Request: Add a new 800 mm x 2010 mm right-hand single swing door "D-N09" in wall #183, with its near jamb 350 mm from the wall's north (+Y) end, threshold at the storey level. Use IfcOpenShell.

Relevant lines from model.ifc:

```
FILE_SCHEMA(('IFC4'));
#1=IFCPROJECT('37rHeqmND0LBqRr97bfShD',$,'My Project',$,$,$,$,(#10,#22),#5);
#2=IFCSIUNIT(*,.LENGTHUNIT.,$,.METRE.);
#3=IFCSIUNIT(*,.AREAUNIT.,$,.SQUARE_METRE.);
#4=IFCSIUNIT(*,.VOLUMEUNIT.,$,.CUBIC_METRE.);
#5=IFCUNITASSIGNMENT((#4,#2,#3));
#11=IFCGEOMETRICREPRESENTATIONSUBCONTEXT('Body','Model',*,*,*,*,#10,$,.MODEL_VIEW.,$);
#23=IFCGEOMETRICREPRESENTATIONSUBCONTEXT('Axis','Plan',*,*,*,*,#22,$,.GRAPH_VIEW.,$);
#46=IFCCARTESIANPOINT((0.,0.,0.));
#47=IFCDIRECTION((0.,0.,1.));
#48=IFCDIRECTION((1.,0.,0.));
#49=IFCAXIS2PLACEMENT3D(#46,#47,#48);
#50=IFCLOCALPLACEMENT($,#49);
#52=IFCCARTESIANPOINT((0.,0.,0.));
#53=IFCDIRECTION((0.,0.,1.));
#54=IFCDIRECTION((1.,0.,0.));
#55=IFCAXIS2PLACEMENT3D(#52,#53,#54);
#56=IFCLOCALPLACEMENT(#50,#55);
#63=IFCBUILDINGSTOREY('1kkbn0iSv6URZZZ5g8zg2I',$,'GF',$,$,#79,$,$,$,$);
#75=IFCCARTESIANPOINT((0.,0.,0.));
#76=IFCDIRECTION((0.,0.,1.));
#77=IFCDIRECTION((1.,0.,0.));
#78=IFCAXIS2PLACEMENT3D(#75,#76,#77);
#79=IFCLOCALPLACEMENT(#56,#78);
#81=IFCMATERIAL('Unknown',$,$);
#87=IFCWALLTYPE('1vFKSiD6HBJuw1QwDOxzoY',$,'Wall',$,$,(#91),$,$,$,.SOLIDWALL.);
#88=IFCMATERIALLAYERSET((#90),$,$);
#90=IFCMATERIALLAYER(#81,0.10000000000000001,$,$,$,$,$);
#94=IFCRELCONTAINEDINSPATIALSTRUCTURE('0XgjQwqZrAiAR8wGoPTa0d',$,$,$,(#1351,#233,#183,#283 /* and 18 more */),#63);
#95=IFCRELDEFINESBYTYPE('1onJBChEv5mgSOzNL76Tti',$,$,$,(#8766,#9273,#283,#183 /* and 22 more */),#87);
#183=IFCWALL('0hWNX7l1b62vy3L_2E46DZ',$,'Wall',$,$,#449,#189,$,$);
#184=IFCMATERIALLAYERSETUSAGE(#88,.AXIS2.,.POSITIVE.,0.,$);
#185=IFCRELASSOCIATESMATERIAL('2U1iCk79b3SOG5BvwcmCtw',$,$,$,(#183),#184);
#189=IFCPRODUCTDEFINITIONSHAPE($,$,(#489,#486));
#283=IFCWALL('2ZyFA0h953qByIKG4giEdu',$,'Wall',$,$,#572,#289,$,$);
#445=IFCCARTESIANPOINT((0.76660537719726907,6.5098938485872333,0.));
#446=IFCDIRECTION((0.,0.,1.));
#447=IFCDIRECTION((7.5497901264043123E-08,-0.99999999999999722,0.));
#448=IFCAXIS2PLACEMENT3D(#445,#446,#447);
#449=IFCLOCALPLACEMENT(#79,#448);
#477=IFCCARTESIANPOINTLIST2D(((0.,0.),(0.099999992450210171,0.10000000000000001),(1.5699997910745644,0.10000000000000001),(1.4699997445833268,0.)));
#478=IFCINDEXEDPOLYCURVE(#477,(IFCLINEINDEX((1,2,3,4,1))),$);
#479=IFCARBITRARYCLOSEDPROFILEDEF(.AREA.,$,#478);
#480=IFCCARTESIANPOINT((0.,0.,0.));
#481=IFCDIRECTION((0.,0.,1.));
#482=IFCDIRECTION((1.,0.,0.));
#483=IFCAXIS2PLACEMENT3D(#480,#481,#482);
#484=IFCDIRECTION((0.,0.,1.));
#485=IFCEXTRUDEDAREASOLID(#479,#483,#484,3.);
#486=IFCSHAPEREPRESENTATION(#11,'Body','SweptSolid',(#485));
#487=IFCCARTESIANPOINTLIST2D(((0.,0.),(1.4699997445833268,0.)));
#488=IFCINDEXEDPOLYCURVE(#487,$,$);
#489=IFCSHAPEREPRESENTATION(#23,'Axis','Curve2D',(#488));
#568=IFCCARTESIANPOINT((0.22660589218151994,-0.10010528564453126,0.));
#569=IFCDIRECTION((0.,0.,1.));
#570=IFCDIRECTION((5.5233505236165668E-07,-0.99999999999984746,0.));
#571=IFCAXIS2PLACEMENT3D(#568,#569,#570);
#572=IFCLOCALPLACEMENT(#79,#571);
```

```python
import numpy as np
import ifcopenshell
import ifcopenshell.api.feature
import ifcopenshell.api.geometry
import ifcopenshell.api.root
import ifcopenshell.api.spatial
import ifcopenshell.geom
import ifcopenshell.util.element
import ifcopenshell.util.placement
import ifcopenshell.util.representation
import ifcopenshell.util.shape
import ifcopenshell.util.unit

model = ifcopenshell.open("model.ifc")
unit_scale = ifcopenshell.util.unit.calculate_unit_scale(model)
settings = ifcopenshell.geom.settings()


def volume(element):
    """Net volume in cubic metres, openings subtracted."""
    shape = ifcopenshell.geom.create_shape(settings, element)
    return ifcopenshell.util.shape.get_volume(shape.geometry)


wall = model.by_id(183)
storey = ifcopenshell.util.element.get_container(wall, ifc_class="IfcBuildingStorey")
context = ifcopenshell.util.representation.get_context(model, "Model", "Body", "MODEL_VIEW")
before = volume(wall)

width, height, from_end, sill = 0.8, 2.01, 0.35, 0.0  # metres

# The wall runs along its own X axis, and the end named is its -X end.
wall_shape = ifcopenshell.geom.create_shape(settings, wall)
x, y, z = ifcopenshell.util.shape.get_vertices(wall_shape.geometry).T
start = x.min() + from_end
face, thickness = float(y.min()), float(y.max() - y.min())
wall_matrix = ifcopenshell.util.placement.get_local_placement(wall.ObjectPlacement)
level = ifcopenshell.util.placement.get_local_placement(storey.ObjectPlacement)[2, 3]


def in_wall(x, y):
    """Placement at x, y metres in the wall's axes, at sill height."""
    matrix = wall_matrix.copy()
    matrix[:, 3] = wall_matrix @ np.array([x / unit_scale, y / unit_scale, 0.0, 1.0])
    matrix[2, 3] = level + sill / unit_scale
    return matrix


# Opening: a box that overshoots both wall faces by 50 mm.
opening = ifcopenshell.api.root.create_entity(model, ifc_class="IfcOpeningElement", predefined_type="OPENING")
box = ifcopenshell.api.geometry.add_wall_representation(
    model, context=context, length=width, height=height, thickness=thickness + 0.1
)
ifcopenshell.api.geometry.assign_representation(model, product=opening, representation=box)
ifcopenshell.api.geometry.edit_object_placement(model, product=opening, matrix=in_wall(start, face - 0.05), is_si=False)
ifcopenshell.api.feature.add_feature(model, feature=opening, element=wall)

door = ifcopenshell.api.root.create_entity(model, ifc_class="IfcDoor", name="D-N09", predefined_type="DOOR")
door.OverallWidth, door.OverallHeight = width / unit_scale, height / unit_scale
door.OperationType = "SINGLE_SWING_RIGHT"
body = ifcopenshell.api.geometry.add_door_representation(
    model,
    context=context,
    overall_width=door.OverallWidth,
    overall_height=door.OverallHeight,
    operation_type="SINGLE_SWING_RIGHT",
    lining_properties={"LiningDepth": thickness / unit_scale, "ThresholdDepth": thickness / unit_scale},
)
ifcopenshell.api.geometry.assign_representation(model, product=door, representation=body)
ifcopenshell.api.spatial.assign_container(model, products=[door], relating_structure=storey)
ifcopenshell.api.feature.add_filling(model, opening=opening, element=door)

# The lining spans the wall, so the door starts at the wall face.
ifcopenshell.api.geometry.edit_object_placement(model, product=door, matrix=in_wall(start, face), is_si=False)

after = volume(wall)

print(f"wall volume {before:.3f} -> {after:.3f} m3")

model.write("model-out.ifc")
```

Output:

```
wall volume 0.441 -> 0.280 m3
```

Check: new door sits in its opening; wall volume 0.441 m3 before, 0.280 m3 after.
